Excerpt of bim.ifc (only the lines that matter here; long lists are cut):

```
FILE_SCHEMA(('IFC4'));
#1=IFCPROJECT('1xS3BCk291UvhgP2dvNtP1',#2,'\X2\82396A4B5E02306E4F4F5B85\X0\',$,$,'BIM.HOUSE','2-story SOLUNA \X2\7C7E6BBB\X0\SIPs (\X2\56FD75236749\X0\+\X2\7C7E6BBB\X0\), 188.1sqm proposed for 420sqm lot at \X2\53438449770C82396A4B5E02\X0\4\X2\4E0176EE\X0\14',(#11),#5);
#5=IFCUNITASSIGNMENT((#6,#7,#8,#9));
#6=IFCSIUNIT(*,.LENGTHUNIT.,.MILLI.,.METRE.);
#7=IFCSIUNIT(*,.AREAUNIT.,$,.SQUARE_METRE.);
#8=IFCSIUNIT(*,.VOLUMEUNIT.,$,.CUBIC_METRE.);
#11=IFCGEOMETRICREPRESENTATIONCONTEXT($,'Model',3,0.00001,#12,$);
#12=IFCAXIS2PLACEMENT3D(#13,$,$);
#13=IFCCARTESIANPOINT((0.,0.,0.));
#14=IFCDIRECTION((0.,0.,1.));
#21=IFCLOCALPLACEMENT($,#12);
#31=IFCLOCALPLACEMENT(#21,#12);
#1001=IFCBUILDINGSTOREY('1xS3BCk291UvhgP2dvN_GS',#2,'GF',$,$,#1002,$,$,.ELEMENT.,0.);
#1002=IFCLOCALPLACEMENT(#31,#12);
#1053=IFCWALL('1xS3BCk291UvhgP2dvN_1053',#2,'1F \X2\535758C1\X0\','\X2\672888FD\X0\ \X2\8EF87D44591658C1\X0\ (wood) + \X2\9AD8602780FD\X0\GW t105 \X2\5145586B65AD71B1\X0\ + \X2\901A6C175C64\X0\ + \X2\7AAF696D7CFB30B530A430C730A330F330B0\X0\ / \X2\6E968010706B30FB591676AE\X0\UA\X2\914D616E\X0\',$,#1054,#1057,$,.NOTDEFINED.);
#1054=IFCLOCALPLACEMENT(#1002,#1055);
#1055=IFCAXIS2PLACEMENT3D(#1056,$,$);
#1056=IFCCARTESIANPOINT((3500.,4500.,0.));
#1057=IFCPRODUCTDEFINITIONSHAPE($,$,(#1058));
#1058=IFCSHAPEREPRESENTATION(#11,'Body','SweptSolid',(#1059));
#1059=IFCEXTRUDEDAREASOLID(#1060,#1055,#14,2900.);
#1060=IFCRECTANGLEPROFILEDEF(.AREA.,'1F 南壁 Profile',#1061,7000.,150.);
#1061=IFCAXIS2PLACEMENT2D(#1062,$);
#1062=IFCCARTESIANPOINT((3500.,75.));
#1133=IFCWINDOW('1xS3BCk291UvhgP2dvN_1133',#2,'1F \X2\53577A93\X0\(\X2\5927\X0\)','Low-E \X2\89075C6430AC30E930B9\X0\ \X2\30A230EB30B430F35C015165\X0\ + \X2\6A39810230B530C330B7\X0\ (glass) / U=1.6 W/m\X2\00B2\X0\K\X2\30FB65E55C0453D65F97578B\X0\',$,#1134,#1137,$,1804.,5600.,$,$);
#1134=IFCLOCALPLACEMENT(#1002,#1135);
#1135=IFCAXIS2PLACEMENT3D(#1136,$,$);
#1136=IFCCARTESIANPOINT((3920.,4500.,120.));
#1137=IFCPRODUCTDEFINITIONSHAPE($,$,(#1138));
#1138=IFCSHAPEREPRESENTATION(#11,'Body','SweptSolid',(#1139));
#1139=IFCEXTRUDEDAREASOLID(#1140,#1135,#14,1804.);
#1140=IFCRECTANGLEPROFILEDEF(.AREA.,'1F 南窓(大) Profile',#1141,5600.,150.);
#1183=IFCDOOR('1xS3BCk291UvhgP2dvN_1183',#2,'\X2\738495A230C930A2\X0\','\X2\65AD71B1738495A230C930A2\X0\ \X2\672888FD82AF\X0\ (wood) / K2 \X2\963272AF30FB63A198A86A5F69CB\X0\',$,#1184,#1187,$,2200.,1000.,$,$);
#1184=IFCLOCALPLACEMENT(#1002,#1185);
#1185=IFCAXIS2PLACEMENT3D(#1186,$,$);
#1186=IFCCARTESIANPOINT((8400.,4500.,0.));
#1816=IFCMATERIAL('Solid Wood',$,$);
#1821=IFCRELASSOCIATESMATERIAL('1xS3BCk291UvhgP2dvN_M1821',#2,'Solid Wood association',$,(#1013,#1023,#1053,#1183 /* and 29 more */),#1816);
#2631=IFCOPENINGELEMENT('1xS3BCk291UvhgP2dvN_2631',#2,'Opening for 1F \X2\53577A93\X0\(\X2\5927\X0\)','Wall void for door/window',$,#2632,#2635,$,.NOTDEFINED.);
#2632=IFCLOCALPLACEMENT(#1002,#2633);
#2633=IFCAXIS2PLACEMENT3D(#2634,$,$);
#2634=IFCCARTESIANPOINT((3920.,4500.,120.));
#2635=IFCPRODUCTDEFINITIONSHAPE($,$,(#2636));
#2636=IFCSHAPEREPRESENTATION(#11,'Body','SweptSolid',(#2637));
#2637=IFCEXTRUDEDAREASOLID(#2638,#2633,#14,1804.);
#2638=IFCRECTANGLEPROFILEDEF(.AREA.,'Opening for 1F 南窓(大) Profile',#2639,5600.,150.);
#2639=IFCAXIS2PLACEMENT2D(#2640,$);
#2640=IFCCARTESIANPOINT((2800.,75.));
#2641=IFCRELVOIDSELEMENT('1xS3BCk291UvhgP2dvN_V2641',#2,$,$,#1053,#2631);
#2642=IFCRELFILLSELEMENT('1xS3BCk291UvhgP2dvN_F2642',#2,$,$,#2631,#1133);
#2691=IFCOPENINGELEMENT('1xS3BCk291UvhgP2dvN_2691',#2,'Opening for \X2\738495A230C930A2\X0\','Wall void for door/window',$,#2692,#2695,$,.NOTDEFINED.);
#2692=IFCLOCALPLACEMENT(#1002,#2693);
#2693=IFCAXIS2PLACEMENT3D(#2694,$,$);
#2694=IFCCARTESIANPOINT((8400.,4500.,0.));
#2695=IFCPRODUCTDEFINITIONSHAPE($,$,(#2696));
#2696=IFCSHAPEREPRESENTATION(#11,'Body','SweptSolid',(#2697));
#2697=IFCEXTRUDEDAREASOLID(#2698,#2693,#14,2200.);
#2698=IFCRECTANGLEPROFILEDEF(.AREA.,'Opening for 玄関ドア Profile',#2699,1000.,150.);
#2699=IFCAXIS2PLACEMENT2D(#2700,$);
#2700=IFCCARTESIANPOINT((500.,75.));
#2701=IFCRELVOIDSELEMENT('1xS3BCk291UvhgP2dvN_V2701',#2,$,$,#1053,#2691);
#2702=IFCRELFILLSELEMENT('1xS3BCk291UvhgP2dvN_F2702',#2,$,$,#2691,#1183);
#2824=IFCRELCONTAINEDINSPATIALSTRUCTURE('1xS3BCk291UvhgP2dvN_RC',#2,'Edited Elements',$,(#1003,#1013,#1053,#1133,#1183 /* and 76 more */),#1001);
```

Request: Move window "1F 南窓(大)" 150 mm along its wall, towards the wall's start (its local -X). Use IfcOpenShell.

```python
import ifcopenshell
import ifcopenshell.api.geometry
import ifcopenshell.util.placement

model = ifcopenshell.open("bim.ifc")

window = model.by_guid("1xS3BCk291UvhgP2dvN_1133")
opening = window.FillsVoids[0].RelatingOpeningElement
wall = opening.VoidsElements[0].RelatingBuildingElement

wall_matrix = ifcopenshell.util.placement.get_local_placement(wall.ObjectPlacement)
shift = wall_matrix[:3, 0] * -150.0
before = ifcopenshell.util.placement.get_local_placement(window.ObjectPlacement)[:3, 3].copy()

# The window is not placed relative to its opening, so move both.
for product in (opening, window):
    matrix = ifcopenshell.util.placement.get_local_placement(product.ObjectPlacement)
    matrix[:3, 3] += shift
    ifcopenshell.api.geometry.edit_object_placement(model, product=product, matrix=matrix, is_si=False)

after = ifcopenshell.util.placement.get_local_placement(window.ObjectPlacement)[:3, 3]
print("window moved by", (after - before).round(3) + 0.0)

model.write("bim_v2.ifc")
```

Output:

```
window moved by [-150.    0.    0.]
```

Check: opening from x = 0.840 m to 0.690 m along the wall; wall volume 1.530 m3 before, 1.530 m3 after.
